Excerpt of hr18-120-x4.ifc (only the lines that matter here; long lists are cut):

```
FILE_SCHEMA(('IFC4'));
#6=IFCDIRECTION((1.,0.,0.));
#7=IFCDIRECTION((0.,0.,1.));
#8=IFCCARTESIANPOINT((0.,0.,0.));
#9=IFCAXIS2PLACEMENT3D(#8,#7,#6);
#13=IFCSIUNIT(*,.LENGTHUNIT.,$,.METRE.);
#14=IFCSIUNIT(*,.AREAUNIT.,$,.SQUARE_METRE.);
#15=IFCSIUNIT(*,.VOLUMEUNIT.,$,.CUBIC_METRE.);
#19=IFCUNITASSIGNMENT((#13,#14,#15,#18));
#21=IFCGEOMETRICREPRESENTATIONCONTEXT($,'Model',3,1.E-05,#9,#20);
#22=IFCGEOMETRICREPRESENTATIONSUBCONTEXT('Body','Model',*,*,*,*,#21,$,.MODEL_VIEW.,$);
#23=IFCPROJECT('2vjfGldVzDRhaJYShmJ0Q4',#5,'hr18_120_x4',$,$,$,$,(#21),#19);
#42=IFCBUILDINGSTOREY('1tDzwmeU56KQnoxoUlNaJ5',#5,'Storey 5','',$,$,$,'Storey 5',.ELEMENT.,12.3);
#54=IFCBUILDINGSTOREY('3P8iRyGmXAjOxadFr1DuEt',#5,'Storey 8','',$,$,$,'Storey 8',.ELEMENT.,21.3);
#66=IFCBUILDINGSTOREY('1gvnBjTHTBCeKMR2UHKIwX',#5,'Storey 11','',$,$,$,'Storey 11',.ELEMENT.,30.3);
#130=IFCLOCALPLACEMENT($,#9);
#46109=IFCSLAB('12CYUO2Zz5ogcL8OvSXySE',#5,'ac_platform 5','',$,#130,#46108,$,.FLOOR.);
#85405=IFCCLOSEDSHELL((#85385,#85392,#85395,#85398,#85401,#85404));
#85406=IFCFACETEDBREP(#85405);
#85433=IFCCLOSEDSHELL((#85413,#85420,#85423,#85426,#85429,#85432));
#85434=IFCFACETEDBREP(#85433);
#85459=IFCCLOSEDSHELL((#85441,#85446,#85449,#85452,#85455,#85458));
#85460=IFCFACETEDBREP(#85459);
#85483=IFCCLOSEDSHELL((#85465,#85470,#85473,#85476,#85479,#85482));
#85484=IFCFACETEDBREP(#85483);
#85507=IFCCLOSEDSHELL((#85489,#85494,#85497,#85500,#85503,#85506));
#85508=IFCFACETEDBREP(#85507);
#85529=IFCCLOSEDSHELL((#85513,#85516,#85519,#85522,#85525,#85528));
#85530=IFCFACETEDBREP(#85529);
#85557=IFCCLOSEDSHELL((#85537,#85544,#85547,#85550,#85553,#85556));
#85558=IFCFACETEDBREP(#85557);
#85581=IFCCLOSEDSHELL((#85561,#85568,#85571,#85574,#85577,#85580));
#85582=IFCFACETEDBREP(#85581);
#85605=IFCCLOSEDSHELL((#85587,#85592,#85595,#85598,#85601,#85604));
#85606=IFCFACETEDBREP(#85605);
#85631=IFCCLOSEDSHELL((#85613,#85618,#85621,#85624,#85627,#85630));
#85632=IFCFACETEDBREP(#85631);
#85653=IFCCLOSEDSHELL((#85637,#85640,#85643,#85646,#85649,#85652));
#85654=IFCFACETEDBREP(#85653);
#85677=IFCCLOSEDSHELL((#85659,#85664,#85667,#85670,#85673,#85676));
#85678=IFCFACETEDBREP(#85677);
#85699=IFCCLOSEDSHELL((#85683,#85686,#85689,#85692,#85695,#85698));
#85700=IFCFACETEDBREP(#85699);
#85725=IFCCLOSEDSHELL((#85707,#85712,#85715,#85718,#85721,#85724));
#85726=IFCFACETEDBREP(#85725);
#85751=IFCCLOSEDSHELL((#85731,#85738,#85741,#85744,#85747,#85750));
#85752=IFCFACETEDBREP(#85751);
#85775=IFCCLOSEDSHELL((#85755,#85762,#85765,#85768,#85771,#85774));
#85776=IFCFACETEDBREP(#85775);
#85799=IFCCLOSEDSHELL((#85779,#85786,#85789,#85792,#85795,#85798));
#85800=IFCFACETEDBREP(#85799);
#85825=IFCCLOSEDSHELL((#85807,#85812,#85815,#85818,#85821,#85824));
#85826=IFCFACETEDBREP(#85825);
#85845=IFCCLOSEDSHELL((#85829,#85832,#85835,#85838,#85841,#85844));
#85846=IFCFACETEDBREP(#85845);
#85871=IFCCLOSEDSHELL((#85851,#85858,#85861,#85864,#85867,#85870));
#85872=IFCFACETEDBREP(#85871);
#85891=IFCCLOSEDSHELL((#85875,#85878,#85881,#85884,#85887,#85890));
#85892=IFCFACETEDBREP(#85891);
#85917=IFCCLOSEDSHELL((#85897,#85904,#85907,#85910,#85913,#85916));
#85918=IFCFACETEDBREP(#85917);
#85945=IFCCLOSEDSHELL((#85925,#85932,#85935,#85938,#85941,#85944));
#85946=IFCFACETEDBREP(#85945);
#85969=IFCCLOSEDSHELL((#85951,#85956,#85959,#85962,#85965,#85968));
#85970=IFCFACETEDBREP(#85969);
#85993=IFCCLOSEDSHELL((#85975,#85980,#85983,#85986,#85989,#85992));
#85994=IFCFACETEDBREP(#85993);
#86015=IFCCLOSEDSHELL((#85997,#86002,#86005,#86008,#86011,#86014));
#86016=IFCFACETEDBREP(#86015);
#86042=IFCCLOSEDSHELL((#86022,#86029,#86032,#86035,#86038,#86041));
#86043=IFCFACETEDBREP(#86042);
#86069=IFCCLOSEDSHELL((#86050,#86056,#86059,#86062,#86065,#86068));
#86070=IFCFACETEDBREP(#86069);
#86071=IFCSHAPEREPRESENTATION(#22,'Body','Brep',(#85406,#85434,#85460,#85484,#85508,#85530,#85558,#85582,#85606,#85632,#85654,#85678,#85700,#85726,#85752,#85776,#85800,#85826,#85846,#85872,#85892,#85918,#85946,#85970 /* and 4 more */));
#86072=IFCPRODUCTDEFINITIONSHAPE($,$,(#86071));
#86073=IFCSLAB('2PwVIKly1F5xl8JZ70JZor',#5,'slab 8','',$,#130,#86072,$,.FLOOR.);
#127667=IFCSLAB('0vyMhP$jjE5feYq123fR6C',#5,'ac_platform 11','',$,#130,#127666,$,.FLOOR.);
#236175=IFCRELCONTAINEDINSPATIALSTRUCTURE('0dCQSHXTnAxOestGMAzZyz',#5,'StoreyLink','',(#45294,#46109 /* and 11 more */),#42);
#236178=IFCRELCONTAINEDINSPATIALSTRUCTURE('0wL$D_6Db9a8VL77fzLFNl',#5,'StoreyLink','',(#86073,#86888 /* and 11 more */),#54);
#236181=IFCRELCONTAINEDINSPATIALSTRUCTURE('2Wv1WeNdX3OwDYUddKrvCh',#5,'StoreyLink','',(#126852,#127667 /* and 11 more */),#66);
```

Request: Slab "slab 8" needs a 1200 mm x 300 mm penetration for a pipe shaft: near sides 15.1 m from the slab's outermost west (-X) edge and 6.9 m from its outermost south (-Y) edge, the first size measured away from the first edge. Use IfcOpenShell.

```python
import numpy as np
import ifcopenshell
import ifcopenshell.api.feature
import ifcopenshell.api.geometry
import ifcopenshell.api.root
import ifcopenshell.geom
import ifcopenshell.util.placement
import ifcopenshell.util.representation
import ifcopenshell.util.shape
import ifcopenshell.util.unit

model = ifcopenshell.open("hr18-120-x4.ifc")
unit_scale = ifcopenshell.util.unit.calculate_unit_scale(model)
settings = ifcopenshell.geom.settings()


def volume(element):
    """Net volume in cubic metres, openings subtracted."""
    shape = ifcopenshell.geom.create_shape(settings, element)
    return ifcopenshell.util.shape.get_volume(shape.geometry)


slab = model.by_guid("2PwVIKly1F5xl8JZ70JZor")
before = volume(slab)

# Extent in the slab's own axes, in metres. The edges named are its -X and -Y sides.
slab_shape = ifcopenshell.geom.create_shape(settings, slab)
vertices = ifcopenshell.util.shape.get_vertices(slab_shape.geometry)
x_min, y_min, bottom = vertices.min(axis=0)
top = vertices[:, 2].max()

opening = ifcopenshell.api.root.create_entity(model, ifc_class="IfcOpeningElement", name="Pipe shaft opening", predefined_type="OPENING")
context = ifcopenshell.util.representation.get_context(model, "Model", "Body", "MODEL_VIEW")
width, depth = 1.2, 0.3
outline = [(0.0, 0.0), (width, 0.0), (width, depth), (0.0, depth), (0.0, 0.0)]
# Overshoot both faces by 50 mm so the cut is clean.
shape = ifcopenshell.api.geometry.add_slab_representation(
    model, context=context, depth=top - bottom + 0.1, polyline=outline
)
ifcopenshell.api.geometry.assign_representation(model, product=opening, representation=shape)

matrix = ifcopenshell.util.placement.get_local_placement(slab.ObjectPlacement)
matrix[:, 3] = matrix @ np.append(np.array([x_min + 15.1, y_min + 6.9, bottom - 0.05]) / unit_scale, 1.0)
ifcopenshell.api.geometry.edit_object_placement(model, product=opening, matrix=matrix, is_si=False)
ifcopenshell.api.feature.add_feature(model, feature=opening, element=slab)

after = volume(slab)

print(f"slab volume {before:.3f} -> {after:.3f} m3")

model.write("hr18-120-x4_v2.ifc")
```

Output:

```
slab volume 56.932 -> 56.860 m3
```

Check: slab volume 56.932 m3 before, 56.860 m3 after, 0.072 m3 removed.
